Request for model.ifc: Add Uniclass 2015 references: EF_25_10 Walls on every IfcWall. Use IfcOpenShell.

First a look at what the model holds.

```python
import ifcopenshell

model = ifcopenshell.open("model.ifc")
print(model.schema)
print("classifications:", [c.Name for c in model.by_type("IfcClassification")])
for ifc_class in ("IfcDoor", "IfcRoof", "IfcStair", "IfcWall", "IfcWindow"):
    print(ifc_class, len(model.by_type(ifc_class)))
```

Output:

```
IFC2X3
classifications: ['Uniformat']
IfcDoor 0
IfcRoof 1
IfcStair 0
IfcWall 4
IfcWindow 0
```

```python
import ifcopenshell
import ifcopenshell.api.classification

model = ifcopenshell.open("model.ifc")

# IFC2X3 requires Source and Edition and has no link from the project to the system.
system = model.create_entity("IfcClassification", Source="NBS", Edition="2015", Name="Uniclass 2015")

codes = {
    "IfcWall": ("EF_25_10", "Walls"),
}
for ifc_class, (code, name) in codes.items():
    products = model.by_type(ifc_class)
    ifcopenshell.api.classification.add_reference(
        model, products=products, classification=system, identification=code, name=name
    )
    print(code, len(products))

model.write("model_rev.ifc")
```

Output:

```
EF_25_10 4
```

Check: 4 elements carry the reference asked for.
